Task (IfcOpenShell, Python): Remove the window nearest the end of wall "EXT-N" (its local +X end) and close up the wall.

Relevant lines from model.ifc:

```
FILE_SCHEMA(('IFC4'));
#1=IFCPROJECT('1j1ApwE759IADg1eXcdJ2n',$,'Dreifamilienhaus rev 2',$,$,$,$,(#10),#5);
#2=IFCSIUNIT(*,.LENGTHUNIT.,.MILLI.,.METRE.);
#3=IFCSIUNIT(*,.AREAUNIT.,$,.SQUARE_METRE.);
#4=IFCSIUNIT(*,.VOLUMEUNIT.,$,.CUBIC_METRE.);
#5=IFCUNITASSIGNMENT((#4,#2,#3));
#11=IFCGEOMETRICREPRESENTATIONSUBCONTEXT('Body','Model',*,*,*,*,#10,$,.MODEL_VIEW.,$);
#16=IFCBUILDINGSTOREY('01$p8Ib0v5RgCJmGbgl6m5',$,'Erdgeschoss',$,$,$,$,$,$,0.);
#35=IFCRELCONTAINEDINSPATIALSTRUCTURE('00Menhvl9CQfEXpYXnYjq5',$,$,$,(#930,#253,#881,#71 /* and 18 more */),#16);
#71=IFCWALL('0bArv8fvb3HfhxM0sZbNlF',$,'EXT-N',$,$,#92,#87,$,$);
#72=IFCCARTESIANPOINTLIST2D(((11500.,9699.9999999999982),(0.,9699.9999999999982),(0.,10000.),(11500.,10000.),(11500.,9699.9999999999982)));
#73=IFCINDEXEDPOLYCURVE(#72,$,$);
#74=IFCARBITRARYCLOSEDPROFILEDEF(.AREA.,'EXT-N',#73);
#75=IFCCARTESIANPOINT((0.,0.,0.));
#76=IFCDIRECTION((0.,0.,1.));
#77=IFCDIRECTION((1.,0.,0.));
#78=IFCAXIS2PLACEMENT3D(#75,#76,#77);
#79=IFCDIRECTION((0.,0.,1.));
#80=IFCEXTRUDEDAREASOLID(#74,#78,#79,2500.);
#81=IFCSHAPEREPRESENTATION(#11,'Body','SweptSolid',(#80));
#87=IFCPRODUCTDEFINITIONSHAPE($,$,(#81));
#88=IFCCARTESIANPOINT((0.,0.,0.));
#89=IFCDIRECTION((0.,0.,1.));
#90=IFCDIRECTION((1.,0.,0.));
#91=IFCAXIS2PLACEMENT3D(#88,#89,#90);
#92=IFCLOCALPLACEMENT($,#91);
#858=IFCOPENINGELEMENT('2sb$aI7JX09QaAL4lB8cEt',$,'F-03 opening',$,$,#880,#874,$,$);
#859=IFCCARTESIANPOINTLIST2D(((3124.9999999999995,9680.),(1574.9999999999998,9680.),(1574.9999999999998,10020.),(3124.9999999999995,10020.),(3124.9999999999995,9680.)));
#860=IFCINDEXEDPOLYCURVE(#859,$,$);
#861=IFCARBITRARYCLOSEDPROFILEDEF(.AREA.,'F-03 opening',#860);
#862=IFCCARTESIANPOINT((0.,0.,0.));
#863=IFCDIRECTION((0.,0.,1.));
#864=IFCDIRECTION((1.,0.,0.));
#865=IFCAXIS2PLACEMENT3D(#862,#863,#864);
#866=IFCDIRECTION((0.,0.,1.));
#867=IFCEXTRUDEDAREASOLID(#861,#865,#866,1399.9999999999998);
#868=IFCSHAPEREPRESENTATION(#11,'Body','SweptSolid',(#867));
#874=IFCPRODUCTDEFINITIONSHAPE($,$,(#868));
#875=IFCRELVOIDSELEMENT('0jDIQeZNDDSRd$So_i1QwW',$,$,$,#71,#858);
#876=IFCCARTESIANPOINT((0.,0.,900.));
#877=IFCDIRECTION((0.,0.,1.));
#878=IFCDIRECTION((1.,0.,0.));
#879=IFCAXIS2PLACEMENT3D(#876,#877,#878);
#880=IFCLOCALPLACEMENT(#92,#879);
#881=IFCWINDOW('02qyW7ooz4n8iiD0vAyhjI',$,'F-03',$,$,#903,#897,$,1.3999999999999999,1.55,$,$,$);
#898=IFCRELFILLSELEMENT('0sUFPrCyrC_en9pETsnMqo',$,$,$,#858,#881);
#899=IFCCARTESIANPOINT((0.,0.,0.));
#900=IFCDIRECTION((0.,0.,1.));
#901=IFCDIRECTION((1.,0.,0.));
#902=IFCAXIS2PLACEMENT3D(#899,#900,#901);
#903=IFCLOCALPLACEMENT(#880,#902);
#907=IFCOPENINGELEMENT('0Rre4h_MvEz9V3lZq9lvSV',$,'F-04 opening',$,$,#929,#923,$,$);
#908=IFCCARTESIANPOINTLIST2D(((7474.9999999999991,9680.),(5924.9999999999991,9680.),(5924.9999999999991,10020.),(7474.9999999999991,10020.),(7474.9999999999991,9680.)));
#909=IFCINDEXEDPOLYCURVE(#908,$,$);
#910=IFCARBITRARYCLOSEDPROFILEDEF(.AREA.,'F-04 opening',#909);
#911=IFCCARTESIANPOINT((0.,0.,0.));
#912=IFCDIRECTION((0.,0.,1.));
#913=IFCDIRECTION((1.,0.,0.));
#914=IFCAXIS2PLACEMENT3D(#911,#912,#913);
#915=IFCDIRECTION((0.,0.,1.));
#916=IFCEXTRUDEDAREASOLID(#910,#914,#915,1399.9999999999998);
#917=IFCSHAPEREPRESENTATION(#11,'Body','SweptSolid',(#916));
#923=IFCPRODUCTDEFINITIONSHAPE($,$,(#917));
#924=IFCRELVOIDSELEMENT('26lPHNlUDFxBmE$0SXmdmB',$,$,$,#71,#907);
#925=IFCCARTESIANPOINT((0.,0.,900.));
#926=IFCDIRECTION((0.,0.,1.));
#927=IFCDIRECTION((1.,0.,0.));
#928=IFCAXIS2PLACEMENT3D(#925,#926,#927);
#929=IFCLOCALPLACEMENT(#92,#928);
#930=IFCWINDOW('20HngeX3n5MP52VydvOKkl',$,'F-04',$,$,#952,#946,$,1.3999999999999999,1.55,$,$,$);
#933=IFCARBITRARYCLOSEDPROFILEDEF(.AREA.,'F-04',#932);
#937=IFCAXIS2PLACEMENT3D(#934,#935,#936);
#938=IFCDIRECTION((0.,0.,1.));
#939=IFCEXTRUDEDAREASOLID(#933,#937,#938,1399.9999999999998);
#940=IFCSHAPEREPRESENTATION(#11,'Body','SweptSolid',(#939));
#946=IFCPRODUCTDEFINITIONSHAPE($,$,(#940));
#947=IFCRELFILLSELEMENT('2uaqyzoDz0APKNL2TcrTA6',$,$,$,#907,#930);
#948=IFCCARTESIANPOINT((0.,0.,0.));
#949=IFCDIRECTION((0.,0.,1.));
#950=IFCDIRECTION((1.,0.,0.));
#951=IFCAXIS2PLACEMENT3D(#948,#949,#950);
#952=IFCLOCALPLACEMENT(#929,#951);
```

```python
import ifcopenshell
import ifcopenshell.api.feature
import ifcopenshell.api.root
import ifcopenshell.geom
import ifcopenshell.util.shape

model = ifcopenshell.open("model.ifc")
settings = ifcopenshell.geom.settings()


def volume(element):
    """Net volume in cubic metres, openings subtracted."""
    shape = ifcopenshell.geom.create_shape(settings, element)
    return ifcopenshell.util.shape.get_volume(shape.geometry)


window = model.by_id(930)
opening = window.FillsVoids[0].RelatingOpeningElement
wall = opening.VoidsElements[0].RelatingBuildingElement
before = volume(wall)

ifcopenshell.api.root.remove_product(model, product=window)
ifcopenshell.api.feature.remove_feature(model, feature=opening)

after = volume(wall)

print(f"wall volume {before:.3f} -> {after:.3f} m3")

model.write("model-out.ifc")
```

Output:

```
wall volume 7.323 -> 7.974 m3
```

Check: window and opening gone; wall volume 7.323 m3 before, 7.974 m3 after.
